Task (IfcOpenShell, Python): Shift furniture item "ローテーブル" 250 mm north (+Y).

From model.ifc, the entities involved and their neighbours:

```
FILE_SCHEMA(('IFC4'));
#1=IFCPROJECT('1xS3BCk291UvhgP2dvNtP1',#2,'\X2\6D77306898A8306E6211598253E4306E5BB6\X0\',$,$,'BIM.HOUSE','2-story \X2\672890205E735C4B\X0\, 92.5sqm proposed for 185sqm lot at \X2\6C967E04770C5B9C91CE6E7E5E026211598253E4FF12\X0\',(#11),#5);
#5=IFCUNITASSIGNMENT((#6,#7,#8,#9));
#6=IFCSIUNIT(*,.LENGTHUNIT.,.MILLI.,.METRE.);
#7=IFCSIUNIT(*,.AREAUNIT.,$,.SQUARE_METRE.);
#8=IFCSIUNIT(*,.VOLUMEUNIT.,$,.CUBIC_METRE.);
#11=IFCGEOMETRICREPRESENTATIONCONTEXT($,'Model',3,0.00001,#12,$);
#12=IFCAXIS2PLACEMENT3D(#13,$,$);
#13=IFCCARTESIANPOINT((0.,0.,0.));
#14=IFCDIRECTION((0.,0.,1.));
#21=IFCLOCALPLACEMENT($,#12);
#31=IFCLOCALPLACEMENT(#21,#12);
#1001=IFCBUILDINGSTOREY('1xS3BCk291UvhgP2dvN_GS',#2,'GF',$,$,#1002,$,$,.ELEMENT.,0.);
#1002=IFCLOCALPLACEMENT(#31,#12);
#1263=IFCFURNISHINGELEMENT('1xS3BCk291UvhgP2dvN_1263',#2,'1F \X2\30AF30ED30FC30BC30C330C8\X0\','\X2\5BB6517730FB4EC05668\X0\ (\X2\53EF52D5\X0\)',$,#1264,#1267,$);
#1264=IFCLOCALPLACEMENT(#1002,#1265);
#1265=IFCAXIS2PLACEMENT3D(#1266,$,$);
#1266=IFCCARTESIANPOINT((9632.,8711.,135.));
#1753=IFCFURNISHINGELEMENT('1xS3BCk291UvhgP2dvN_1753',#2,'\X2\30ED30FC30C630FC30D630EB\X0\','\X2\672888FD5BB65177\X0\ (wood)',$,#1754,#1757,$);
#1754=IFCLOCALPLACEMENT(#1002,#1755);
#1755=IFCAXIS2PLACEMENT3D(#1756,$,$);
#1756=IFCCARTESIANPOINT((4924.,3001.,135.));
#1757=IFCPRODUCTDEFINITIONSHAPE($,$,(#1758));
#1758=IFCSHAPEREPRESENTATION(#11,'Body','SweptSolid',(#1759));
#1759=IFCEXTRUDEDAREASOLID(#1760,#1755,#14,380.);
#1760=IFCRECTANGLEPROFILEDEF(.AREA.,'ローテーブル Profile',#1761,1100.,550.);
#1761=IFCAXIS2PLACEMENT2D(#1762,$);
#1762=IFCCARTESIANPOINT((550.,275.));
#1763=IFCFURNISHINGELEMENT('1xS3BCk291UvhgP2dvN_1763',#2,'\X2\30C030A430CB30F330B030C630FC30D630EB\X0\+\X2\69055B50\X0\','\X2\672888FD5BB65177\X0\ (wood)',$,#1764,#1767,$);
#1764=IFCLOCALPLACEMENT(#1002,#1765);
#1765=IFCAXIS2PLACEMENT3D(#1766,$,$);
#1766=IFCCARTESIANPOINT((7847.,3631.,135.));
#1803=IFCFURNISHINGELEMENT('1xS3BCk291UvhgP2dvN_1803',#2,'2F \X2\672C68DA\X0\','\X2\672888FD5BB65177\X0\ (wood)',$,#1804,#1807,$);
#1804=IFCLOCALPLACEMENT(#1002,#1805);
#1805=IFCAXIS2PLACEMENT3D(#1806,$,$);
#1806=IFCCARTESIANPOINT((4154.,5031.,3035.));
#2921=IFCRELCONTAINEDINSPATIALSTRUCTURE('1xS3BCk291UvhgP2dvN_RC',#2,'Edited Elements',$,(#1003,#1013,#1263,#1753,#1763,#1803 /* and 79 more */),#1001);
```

```python
import ifcopenshell
import ifcopenshell.api.geometry
import ifcopenshell.util.placement
import ifcopenshell.util.unit

model = ifcopenshell.open("model.ifc")
unit_scale = ifcopenshell.util.unit.calculate_unit_scale(model)

item = model.by_guid("1xS3BCk291UvhgP2dvN_1753")
matrix = ifcopenshell.util.placement.get_local_placement(item.ObjectPlacement)
matrix[1, 3] += 0.25 / unit_scale
ifcopenshell.api.geometry.edit_object_placement(model, product=item, matrix=matrix, is_si=False)

print(ifcopenshell.util.placement.get_local_placement(item.ObjectPlacement).round(3) + 0.0)

model.write("model_edited.ifc")
```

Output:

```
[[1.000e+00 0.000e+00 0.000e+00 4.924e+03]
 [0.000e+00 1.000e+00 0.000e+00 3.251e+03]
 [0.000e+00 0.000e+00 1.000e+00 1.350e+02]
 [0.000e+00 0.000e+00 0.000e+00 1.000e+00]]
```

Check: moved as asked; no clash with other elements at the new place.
